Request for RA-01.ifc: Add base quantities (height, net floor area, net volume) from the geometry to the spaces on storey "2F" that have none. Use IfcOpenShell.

First a look at what the model holds.

```python
import ifcopenshell
import ifcopenshell.util.element
import ifcopenshell.util.unit

model = ifcopenshell.open("RA-01.ifc")
print(model.schema)
for unit_type in ("LENGTHUNIT", "AREAUNIT", "VOLUMEUNIT"):
    print(unit_type, ifcopenshell.util.unit.calculate_unit_scale(model, unit_type))
storey = next(s for s in model.by_type("IfcBuildingStorey") if s.Name == "2F")
spaces = [e for e in ifcopenshell.util.element.get_decomposition(storey) if e.is_a("IfcSpace")]
for e in sorted(spaces, key=lambda e: e.id()):
    print(e.id(), e.is_a(), e.Name, list(ifcopenshell.util.element.get_psets(e, qtos_only=True)), sep=" | ")
```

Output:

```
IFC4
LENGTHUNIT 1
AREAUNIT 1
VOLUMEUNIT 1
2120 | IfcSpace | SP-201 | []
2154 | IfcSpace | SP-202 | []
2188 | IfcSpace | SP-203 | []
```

```python
import ifcopenshell
import ifcopenshell.api.pset
import ifcopenshell.geom
import ifcopenshell.util.element
import ifcopenshell.util.shape
import ifcopenshell.util.unit

model = ifcopenshell.open("RA-01.ifc")
unit_scale = ifcopenshell.util.unit.calculate_unit_scale(model)
area_scale = ifcopenshell.util.unit.calculate_unit_scale(model, "AREAUNIT")
volume_scale = ifcopenshell.util.unit.calculate_unit_scale(model, "VOLUMEUNIT")
settings = ifcopenshell.geom.settings()

storey = next(s for s in model.by_type("IfcBuildingStorey") if s.Name == "2F")
spaces = [e for e in ifcopenshell.util.element.get_decomposition(storey) if e.is_a("IfcSpace")]

for e in sorted(spaces, key=lambda e: e.id()):
    if ifcopenshell.util.element.get_psets(e, qtos_only=True, should_inherit=False):
        continue
    # Geometry comes back in metres, in the element's own axes.
    shape = ifcopenshell.geom.create_shape(settings, e)
    values = {
        "Height": ifcopenshell.util.shape.get_z(shape.geometry) / unit_scale,
        "NetFloorArea": ifcopenshell.util.shape.get_footprint_area(shape.geometry) / area_scale,
        "NetVolume": ifcopenshell.util.shape.get_volume(shape.geometry) / volume_scale,
    }
    qto = ifcopenshell.api.pset.add_qto(model, product=e, name="Qto_SpaceBaseQuantities")
    ifcopenshell.api.pset.edit_qto(model, qto=qto, properties=values)
    print(e.id(), {k: round(v, 3) for k, v in values.items()})

model.write("RA-01-out.ifc")
```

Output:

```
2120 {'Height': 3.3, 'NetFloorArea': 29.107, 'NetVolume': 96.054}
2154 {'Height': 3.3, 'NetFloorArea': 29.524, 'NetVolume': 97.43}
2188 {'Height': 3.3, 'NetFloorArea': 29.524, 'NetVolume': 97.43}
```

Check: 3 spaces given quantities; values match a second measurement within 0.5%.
